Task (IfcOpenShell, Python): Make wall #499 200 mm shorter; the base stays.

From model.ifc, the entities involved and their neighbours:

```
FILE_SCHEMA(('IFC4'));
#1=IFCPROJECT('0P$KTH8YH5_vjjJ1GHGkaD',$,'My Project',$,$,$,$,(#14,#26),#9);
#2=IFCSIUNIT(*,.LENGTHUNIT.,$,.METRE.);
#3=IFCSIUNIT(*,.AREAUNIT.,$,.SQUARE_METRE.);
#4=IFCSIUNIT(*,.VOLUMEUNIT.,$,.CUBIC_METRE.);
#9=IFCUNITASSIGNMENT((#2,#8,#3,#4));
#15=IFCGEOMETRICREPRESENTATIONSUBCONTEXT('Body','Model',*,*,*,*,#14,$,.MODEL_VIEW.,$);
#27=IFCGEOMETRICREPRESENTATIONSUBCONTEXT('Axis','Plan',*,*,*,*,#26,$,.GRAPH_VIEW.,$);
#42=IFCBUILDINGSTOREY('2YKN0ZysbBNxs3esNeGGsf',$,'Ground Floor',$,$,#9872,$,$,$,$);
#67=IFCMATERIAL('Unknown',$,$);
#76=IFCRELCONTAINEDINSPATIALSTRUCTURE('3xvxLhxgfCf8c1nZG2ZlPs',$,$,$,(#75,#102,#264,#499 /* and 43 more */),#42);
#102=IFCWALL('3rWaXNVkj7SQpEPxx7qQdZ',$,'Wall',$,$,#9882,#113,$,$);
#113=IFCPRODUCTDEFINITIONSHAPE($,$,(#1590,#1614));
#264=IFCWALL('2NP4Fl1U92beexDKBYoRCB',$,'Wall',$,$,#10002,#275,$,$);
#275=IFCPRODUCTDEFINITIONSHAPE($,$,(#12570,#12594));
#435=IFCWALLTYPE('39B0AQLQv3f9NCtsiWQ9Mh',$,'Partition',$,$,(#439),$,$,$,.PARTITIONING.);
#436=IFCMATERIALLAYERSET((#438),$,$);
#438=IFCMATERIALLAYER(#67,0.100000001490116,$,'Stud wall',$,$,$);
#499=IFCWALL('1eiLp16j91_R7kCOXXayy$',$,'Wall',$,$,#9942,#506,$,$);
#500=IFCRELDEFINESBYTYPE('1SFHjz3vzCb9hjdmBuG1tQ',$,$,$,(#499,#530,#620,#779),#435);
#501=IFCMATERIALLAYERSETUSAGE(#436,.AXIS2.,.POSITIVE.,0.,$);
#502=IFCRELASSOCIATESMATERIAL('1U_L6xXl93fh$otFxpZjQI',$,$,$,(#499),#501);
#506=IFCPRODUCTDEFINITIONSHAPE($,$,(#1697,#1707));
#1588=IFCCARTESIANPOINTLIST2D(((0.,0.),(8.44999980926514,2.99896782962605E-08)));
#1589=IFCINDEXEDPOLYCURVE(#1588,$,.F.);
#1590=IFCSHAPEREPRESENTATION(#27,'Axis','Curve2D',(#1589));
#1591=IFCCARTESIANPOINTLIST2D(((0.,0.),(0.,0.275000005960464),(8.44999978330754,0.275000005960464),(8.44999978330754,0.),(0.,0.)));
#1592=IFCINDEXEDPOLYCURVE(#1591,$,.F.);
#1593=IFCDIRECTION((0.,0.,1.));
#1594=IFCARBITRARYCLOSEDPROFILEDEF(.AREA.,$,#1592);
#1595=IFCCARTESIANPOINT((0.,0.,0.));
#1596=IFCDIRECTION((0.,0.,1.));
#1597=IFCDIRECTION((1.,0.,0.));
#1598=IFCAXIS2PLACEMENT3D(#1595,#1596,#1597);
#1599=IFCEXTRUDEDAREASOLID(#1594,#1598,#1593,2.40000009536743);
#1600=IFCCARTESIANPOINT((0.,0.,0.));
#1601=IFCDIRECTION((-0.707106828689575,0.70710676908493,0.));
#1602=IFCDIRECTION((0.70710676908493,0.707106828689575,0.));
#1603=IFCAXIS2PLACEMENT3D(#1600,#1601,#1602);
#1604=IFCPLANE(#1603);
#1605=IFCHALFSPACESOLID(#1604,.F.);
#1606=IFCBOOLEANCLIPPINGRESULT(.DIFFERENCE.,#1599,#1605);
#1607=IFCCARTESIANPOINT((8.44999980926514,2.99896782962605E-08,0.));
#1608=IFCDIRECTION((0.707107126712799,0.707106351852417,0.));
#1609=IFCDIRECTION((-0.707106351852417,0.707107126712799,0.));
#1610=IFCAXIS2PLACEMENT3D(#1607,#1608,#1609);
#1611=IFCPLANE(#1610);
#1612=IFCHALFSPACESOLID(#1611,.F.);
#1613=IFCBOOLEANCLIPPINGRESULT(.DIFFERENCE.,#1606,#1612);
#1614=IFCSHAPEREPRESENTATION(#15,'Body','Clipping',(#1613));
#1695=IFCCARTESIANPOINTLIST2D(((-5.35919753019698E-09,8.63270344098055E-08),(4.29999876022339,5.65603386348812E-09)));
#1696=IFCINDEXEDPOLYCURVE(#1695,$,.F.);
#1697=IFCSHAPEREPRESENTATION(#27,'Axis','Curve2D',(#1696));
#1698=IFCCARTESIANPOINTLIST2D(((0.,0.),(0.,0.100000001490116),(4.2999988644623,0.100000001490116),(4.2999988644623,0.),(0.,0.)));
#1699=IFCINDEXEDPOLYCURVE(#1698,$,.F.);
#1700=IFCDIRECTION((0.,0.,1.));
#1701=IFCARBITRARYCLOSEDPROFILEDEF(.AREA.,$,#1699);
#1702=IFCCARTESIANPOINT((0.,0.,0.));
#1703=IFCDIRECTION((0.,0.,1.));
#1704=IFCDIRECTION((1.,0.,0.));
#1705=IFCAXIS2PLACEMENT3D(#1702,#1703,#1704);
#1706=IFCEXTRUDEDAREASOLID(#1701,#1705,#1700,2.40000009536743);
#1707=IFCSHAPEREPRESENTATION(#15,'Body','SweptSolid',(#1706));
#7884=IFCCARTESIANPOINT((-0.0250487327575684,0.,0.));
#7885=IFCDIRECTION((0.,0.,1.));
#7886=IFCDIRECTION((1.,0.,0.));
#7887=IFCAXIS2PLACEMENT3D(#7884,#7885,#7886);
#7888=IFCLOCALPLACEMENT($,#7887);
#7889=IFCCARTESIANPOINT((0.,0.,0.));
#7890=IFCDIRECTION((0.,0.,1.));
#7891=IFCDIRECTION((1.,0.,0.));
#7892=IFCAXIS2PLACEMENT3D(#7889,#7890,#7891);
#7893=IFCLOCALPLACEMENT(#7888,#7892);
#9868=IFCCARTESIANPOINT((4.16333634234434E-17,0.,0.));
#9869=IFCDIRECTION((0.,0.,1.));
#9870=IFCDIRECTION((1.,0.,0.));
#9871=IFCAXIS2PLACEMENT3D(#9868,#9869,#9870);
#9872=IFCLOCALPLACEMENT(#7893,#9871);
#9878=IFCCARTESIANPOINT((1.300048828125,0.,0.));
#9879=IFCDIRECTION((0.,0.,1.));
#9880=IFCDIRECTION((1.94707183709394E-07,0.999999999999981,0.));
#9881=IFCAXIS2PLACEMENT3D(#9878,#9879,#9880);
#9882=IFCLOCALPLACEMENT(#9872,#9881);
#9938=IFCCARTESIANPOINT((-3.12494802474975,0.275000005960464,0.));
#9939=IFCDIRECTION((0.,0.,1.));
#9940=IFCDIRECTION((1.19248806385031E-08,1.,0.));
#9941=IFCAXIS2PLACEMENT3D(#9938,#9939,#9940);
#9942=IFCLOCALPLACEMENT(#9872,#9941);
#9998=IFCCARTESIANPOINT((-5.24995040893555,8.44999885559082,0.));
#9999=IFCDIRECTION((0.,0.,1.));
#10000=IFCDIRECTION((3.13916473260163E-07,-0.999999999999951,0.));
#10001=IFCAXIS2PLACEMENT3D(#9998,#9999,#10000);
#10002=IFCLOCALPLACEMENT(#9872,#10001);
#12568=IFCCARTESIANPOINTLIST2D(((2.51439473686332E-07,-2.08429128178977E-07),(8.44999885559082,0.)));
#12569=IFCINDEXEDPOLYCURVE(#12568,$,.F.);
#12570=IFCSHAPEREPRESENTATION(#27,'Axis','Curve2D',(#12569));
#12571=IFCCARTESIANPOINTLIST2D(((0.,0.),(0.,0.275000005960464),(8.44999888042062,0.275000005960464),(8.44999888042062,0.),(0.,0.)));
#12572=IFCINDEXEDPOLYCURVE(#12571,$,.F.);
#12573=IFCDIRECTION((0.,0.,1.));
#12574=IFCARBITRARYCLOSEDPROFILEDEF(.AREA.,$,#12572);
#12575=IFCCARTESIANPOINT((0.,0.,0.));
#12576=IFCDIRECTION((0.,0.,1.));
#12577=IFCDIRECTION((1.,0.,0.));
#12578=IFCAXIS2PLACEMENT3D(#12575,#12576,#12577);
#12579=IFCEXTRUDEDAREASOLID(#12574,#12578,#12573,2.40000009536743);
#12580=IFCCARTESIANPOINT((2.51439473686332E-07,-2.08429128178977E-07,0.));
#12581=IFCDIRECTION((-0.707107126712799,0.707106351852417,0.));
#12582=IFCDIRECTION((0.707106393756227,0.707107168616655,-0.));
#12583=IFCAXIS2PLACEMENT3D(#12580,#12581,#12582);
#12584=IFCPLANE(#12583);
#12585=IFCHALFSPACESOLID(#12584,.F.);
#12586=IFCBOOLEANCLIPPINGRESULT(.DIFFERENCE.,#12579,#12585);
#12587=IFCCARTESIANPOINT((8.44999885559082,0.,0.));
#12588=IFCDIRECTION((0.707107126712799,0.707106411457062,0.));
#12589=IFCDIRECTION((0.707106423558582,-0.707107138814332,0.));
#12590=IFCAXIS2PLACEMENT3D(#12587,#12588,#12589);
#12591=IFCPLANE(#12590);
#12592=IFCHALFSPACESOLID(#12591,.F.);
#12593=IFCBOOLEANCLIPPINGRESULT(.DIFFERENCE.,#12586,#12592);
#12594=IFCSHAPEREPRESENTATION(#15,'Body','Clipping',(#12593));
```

```python
import ifcopenshell
import ifcopenshell.geom
import ifcopenshell.util.representation
import ifcopenshell.util.shape
import ifcopenshell.util.unit

model = ifcopenshell.open("model.ifc")
unit_scale = ifcopenshell.util.unit.calculate_unit_scale(model)
settings = ifcopenshell.geom.settings()


def volume(element):
    """Net volume in cubic metres, openings subtracted."""
    shape = ifcopenshell.geom.create_shape(settings, element)
    return ifcopenshell.util.shape.get_volume(shape.geometry)


wall = model.by_id(499)
before = volume(wall)

body = ifcopenshell.util.representation.get_representation(wall, "Model", "Body")
solid = body.Items[0]
old_height = solid.Depth
solid.Depth -= 0.2 / unit_scale
after = volume(wall)

print(f"height {old_height:g} -> {solid.Depth:g}, volume {before:.3f} -> {after:.3f} m3")

model.write("model-out.ifc")
```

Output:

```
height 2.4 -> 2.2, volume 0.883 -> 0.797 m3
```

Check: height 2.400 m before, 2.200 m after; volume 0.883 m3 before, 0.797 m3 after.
